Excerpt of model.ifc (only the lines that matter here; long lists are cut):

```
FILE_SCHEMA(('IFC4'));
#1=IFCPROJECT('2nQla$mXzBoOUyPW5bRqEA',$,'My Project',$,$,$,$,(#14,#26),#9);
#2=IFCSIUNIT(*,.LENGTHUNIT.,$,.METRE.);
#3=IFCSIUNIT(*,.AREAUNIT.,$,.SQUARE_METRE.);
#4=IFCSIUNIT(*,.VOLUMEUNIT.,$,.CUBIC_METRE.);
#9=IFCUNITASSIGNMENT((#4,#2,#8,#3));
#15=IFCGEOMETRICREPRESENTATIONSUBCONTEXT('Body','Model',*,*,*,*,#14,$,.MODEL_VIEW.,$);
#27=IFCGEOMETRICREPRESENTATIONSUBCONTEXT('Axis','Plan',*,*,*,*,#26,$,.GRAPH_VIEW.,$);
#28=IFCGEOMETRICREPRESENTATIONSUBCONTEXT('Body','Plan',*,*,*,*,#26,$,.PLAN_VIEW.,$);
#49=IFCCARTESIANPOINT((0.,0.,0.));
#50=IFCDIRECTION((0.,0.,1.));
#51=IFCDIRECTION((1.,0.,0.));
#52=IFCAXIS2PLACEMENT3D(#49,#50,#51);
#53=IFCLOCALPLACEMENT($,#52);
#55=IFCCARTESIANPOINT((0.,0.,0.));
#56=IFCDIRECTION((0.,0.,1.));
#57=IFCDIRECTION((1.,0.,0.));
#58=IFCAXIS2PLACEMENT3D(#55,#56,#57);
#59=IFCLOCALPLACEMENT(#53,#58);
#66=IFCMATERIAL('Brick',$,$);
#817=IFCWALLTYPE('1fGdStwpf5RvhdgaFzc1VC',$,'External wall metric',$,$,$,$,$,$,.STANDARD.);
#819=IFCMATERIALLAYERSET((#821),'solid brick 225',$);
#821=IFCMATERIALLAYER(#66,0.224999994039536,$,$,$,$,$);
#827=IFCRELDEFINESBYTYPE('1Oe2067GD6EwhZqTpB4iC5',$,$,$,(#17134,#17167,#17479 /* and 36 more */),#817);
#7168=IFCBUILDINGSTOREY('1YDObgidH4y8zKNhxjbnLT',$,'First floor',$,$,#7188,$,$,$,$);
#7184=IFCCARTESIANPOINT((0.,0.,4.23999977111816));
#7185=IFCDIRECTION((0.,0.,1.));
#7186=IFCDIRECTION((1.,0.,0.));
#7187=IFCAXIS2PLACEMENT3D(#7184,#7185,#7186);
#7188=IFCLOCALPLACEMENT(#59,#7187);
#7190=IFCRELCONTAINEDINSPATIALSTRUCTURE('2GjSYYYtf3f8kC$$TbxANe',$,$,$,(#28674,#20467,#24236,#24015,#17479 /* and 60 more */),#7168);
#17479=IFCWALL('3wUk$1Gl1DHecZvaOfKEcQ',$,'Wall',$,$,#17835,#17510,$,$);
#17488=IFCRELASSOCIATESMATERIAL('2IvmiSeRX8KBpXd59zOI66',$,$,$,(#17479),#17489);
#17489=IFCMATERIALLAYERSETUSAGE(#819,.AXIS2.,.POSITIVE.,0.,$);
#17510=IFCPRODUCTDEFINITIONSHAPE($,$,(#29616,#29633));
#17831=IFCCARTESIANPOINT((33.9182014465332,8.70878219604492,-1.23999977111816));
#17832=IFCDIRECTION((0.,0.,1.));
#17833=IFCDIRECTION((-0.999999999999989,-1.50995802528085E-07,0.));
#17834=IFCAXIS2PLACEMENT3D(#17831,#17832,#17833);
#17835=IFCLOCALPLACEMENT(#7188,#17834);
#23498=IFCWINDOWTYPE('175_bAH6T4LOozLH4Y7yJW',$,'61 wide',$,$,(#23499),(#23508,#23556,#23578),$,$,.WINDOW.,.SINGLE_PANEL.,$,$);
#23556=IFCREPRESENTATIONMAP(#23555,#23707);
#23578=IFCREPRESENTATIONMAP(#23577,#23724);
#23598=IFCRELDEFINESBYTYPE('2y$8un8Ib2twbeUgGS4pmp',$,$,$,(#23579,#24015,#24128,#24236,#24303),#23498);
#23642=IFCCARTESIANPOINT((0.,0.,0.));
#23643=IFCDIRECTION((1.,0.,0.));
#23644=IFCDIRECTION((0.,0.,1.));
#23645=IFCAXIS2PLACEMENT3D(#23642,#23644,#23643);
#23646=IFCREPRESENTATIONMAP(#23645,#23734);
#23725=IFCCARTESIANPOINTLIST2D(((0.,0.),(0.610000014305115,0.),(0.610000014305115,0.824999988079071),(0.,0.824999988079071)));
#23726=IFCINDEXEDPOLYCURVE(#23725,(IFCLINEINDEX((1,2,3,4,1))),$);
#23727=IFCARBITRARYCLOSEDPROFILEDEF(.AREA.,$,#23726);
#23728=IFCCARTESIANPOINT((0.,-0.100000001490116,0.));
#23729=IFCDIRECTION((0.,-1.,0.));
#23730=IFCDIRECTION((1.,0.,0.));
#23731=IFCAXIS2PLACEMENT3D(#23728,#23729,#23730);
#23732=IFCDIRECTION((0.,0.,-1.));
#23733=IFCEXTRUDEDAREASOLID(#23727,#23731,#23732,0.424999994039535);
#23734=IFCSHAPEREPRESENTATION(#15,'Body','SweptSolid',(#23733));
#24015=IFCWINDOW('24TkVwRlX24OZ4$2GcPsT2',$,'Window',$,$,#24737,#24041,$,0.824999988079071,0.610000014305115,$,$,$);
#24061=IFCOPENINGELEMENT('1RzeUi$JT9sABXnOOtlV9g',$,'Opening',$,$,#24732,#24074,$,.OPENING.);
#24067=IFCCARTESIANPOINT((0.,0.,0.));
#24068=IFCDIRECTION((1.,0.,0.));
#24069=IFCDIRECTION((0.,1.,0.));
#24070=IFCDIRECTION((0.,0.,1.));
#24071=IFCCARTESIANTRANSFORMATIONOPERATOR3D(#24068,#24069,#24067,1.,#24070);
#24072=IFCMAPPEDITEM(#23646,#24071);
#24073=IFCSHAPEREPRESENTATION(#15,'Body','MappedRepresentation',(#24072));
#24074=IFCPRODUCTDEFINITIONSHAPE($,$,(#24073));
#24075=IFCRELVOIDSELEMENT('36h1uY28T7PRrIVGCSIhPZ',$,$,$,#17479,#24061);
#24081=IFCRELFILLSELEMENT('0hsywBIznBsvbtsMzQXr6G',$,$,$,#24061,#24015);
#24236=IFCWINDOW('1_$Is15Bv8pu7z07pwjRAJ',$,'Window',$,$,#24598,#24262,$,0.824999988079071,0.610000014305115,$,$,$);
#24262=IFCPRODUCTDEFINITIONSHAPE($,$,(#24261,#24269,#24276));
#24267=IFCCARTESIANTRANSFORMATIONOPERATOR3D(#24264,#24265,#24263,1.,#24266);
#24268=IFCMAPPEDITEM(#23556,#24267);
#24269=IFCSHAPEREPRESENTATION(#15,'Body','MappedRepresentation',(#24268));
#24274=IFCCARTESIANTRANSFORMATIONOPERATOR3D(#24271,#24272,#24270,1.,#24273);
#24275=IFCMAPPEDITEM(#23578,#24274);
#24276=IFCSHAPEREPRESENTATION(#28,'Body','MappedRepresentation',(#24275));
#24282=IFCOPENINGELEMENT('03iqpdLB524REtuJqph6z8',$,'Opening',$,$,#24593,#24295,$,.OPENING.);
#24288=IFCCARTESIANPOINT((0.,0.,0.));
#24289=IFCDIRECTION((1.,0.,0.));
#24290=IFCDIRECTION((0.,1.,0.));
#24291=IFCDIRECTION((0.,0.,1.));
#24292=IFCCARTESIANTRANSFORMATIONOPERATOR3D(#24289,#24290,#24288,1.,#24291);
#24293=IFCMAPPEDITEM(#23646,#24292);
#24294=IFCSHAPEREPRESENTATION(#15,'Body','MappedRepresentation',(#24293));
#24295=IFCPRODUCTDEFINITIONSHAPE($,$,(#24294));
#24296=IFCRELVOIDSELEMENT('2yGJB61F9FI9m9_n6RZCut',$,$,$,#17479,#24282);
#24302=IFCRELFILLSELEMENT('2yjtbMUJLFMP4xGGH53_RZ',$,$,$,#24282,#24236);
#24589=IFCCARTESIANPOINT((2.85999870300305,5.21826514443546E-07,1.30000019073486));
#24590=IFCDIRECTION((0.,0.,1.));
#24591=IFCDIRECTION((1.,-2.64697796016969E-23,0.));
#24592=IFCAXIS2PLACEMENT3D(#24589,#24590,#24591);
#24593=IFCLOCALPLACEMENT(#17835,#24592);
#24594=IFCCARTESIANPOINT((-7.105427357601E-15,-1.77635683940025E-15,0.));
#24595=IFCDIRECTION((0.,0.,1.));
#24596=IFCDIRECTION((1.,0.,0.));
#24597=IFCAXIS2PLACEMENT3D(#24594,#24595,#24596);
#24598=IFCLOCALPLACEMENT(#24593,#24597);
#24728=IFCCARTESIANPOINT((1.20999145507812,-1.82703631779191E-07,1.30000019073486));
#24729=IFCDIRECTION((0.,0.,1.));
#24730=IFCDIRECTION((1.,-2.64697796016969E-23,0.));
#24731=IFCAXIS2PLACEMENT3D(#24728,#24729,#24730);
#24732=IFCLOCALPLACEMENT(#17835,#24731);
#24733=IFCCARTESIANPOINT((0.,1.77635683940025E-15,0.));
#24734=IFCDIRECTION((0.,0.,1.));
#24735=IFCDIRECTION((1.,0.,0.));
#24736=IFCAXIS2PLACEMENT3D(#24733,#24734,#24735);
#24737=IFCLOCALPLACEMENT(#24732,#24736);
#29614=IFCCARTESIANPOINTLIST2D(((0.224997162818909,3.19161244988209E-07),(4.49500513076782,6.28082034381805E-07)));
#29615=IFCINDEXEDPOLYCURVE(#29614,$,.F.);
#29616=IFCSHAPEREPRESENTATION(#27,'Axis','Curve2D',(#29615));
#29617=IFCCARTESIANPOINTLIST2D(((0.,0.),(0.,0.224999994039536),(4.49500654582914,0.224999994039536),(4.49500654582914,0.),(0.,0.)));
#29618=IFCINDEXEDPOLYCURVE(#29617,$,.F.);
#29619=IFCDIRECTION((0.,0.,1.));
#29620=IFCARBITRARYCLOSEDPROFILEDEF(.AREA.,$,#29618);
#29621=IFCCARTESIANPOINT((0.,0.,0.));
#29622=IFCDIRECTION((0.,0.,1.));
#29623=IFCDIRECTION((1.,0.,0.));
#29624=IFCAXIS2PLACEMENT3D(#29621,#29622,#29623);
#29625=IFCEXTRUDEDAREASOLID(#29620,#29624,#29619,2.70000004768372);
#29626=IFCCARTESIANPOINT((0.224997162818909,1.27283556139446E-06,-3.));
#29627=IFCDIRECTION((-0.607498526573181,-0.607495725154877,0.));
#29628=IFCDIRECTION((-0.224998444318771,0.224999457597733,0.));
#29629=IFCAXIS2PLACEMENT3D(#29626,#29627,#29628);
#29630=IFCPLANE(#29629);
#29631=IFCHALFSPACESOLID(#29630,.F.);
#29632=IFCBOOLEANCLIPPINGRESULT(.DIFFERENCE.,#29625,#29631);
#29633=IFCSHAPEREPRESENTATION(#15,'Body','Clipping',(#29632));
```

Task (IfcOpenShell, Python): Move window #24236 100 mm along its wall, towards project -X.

```python
import ifcopenshell
import ifcopenshell.api.geometry
import ifcopenshell.util.placement
import ifcopenshell.util.unit

model = ifcopenshell.open("model.ifc")
unit_scale = ifcopenshell.util.unit.calculate_unit_scale(model)

window = model.by_id(24236)
opening = window.FillsVoids[0].RelatingOpeningElement
wall = opening.VoidsElements[0].RelatingBuildingElement

wall_matrix = ifcopenshell.util.placement.get_local_placement(wall.ObjectPlacement)
shift = wall_matrix[:3, 0] * 0.1 / unit_scale
before = ifcopenshell.util.placement.get_local_placement(window.ObjectPlacement)[:3, 3].copy()

# The window is placed relative to its opening, so it follows when the opening moves.
matrix = ifcopenshell.util.placement.get_local_placement(opening.ObjectPlacement)
matrix[:3, 3] += shift
ifcopenshell.api.geometry.edit_object_placement(
    model, product=opening, matrix=matrix, is_si=False, should_transform_children=True
)

after = ifcopenshell.util.placement.get_local_placement(window.ObjectPlacement)[:3, 3]
print("window moved by", (after - before).round(3) + 0.0)

model.write("model_rev.ifc")
```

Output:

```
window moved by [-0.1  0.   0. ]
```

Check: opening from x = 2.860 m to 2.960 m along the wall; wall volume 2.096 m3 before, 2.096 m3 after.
